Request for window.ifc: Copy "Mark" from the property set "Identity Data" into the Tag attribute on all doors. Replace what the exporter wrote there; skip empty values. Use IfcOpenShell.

First a look at what the model holds.

```python
import ifcopenshell
import ifcopenshell.util.element

model = ifcopenshell.open("window.ifc")
print(model.schema)
doors = model.by_type("IfcDoor")
print(len(doors), "doors")
for e in doors[:8]:
    source = ifcopenshell.util.element.get_pset(e, "Identity Data", "Mark")
    target = e.Tag
    print(e.id(), repr(source), repr(target), sep=" | ")
```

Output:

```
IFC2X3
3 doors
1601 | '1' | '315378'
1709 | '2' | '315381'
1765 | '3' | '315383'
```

```python
import ifcopenshell
import ifcopenshell.util.element

model = ifcopenshell.open("window.ifc")

count = 0
for e in model.by_type("IfcDoor"):
    value = ifcopenshell.util.element.get_pset(e, "Identity Data", "Mark")
    current = e.Tag
    if not value or not value.strip() or current == value:
        continue
    e.Tag = value
    count += 1

print(count, "doors updated")

model.write("window_updated.ifc")
```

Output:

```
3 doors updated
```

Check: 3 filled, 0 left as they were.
